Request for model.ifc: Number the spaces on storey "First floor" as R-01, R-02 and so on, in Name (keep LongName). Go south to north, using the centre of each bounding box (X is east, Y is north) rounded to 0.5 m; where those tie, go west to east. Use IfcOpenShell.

First a look at what the model holds.

```python
import ifcopenshell
import ifcopenshell.util.element
import ifcopenshell.util.placement

model = ifcopenshell.open("model.ifc")
print(model.schema)
storey = next(s for s in model.by_type("IfcBuildingStorey") if s.Name == "First floor")
spaces = [e for e in ifcopenshell.util.element.get_decomposition(storey) if e.is_a("IfcSpace")]
for e in sorted(spaces, key=lambda e: e.id()):
    origin = ifcopenshell.util.placement.get_local_placement(e.ObjectPlacement)[:3, 3]
    print(e.id(), e.Name, e.LongName, origin.round(2) + 0.0, sep=" | ")
```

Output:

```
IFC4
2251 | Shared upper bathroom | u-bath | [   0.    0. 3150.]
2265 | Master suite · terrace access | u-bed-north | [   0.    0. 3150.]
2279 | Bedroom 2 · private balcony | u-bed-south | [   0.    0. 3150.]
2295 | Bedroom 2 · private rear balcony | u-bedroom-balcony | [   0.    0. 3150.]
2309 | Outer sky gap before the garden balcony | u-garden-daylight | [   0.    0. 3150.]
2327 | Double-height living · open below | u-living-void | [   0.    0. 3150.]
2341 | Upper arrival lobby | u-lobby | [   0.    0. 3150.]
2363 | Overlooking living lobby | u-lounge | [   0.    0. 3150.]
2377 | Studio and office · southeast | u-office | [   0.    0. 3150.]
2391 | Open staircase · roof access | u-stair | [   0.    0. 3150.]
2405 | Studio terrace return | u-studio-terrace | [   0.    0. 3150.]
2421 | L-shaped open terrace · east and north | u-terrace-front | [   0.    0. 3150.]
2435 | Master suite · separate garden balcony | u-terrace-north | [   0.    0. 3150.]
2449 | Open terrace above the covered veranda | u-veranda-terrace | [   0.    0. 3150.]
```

```python
import ifcopenshell
import ifcopenshell.geom
import ifcopenshell.util.element
import ifcopenshell.util.shape

model = ifcopenshell.open("model.ifc")
settings = ifcopenshell.geom.settings()
settings.set("use-world-coords", True)


def centre(element):
    shape = ifcopenshell.geom.create_shape(settings, element)
    return ifcopenshell.util.shape.get_bbox_centroid(shape.geometry)


storey = next(s for s in model.by_type("IfcBuildingStorey") if s.Name == "First floor")
spaces = [e for e in ifcopenshell.util.element.get_decomposition(storey) if e.is_a("IfcSpace")]

# Insertion points can sit at a corner or the storey origin, so sort by the geometry (in metres).
centres = {e: centre(e) for e in spaces}
spaces.sort(key=lambda e: (round(centres[e][1] / 0.5), centres[e][0]))

for i, e in enumerate(spaces, start=1):
    number = f"R-{i:02d}"
    e.Name = number
    print(e.id(), number)

model.write("model-out.ifc")
```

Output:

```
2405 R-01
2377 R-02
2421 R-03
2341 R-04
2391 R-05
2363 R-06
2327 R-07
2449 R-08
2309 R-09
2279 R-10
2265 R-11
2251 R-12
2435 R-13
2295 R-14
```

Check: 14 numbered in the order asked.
